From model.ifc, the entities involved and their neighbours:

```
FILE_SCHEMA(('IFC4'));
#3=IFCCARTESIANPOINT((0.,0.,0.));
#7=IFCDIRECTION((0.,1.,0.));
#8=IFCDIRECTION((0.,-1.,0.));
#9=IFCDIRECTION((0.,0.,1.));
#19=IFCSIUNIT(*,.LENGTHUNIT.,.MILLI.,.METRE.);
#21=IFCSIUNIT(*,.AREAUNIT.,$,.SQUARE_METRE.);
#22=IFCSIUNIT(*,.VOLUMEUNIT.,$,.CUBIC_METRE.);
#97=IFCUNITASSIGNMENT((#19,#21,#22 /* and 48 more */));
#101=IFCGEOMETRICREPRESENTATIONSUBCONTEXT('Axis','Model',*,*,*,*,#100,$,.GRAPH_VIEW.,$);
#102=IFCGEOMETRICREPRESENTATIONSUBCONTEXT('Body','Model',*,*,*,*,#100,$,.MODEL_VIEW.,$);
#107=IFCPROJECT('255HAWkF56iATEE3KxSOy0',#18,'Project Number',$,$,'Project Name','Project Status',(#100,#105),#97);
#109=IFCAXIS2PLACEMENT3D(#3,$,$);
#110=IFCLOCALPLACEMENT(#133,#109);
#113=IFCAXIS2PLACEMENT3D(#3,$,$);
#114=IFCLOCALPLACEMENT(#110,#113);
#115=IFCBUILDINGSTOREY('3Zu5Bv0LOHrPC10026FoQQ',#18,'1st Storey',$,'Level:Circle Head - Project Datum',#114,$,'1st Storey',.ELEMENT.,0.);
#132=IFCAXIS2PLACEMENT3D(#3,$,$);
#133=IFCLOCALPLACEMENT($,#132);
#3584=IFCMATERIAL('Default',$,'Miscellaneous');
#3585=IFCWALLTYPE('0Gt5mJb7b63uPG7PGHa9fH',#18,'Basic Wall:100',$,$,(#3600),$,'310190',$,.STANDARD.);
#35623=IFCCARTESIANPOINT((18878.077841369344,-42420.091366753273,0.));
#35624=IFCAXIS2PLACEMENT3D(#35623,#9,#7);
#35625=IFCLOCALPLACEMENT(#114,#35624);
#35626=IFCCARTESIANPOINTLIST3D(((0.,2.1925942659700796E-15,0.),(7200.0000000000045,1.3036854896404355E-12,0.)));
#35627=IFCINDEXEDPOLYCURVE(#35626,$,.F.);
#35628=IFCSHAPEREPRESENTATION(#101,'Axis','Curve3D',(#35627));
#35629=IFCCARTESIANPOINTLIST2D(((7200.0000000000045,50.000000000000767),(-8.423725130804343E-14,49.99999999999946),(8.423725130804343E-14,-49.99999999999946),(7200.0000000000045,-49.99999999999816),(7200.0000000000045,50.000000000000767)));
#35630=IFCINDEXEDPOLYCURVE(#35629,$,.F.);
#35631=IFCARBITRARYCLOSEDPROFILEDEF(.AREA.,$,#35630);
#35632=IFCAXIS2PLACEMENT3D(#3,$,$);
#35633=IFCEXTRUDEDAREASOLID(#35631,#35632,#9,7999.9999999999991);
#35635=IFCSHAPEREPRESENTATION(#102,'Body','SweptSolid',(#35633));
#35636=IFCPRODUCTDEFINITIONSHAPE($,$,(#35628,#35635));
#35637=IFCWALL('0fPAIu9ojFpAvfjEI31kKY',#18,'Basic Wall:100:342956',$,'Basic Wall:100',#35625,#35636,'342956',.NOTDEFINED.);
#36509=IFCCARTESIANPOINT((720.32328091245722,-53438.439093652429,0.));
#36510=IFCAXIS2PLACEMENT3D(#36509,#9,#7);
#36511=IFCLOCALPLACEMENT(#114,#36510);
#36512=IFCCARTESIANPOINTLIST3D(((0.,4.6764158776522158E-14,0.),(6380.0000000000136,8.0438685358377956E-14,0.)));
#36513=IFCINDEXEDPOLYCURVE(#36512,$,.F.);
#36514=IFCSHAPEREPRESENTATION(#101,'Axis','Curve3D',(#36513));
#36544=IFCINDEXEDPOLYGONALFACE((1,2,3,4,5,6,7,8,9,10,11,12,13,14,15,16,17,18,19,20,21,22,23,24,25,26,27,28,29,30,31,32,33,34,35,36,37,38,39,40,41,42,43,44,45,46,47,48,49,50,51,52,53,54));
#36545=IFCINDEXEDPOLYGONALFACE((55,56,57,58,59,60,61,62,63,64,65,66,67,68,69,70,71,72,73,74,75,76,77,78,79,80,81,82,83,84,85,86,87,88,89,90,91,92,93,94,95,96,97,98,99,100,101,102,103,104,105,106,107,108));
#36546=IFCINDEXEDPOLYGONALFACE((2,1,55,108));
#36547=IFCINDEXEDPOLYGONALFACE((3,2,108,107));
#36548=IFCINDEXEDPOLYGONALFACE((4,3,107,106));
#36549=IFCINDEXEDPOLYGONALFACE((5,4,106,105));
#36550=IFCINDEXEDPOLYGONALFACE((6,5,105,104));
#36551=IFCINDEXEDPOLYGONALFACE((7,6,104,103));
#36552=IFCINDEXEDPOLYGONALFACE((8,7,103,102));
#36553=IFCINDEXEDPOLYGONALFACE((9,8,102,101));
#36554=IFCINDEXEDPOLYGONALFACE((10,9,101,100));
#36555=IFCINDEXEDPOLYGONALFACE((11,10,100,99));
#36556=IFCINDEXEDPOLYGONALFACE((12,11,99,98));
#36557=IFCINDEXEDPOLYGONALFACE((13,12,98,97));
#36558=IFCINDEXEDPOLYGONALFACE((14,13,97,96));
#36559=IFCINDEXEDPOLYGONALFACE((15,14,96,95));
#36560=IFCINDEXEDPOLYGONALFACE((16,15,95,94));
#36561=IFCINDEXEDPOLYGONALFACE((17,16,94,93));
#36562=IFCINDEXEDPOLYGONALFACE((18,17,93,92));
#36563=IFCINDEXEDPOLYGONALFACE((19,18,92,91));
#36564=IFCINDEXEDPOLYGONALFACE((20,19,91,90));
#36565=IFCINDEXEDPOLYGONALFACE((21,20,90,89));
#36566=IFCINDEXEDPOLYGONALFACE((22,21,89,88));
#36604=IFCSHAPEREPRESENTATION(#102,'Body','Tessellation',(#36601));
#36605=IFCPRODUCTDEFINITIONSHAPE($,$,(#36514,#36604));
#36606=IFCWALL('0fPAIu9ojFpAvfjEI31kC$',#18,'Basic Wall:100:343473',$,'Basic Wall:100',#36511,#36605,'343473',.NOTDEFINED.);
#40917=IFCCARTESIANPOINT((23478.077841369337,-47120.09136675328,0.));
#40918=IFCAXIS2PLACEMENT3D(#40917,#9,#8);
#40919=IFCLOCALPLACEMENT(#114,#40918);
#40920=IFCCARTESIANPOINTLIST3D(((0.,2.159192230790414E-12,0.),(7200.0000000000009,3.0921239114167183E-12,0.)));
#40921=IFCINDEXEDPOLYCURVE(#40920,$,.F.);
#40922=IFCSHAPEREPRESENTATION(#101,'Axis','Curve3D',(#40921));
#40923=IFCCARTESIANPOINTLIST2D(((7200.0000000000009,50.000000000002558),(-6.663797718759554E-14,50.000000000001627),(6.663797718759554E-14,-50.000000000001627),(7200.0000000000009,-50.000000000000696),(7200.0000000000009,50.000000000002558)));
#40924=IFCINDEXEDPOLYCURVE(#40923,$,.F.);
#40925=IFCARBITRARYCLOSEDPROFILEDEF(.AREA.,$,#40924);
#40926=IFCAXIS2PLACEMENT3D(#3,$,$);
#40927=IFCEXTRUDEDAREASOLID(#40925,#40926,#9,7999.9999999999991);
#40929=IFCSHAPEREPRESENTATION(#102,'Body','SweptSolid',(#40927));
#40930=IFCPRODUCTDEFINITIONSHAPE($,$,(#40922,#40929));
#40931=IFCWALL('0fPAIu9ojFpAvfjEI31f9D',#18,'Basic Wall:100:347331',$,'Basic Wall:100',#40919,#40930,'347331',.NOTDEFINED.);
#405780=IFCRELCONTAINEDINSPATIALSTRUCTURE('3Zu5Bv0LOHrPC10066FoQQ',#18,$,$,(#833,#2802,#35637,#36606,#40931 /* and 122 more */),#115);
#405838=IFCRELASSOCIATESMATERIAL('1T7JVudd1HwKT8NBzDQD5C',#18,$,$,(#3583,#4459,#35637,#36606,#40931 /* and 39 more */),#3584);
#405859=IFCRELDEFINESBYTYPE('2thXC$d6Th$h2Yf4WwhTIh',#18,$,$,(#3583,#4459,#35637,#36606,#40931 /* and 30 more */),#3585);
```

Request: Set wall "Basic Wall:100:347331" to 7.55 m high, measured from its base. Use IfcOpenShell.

```python
import ifcopenshell
import ifcopenshell.geom
import ifcopenshell.util.representation
import ifcopenshell.util.shape
import ifcopenshell.util.unit

model = ifcopenshell.open("model.ifc")
unit_scale = ifcopenshell.util.unit.calculate_unit_scale(model)
settings = ifcopenshell.geom.settings()


def volume(element):
    """Net volume in cubic metres, openings subtracted."""
    shape = ifcopenshell.geom.create_shape(settings, element)
    return ifcopenshell.util.shape.get_volume(shape.geometry)


wall = model.by_guid("0fPAIu9ojFpAvfjEI31f9D")
before = volume(wall)

body = ifcopenshell.util.representation.get_representation(wall, "Model", "Body")
solid = body.Items[0]
old_height = solid.Depth
solid.Depth = 7.55 / unit_scale
after = volume(wall)

print(f"height {old_height:g} -> {solid.Depth:g}, volume {before:.3f} -> {after:.3f} m3")

model.write("model_updated.ifc")
```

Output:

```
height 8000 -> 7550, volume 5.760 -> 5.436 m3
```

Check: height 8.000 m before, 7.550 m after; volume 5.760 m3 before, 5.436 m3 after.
